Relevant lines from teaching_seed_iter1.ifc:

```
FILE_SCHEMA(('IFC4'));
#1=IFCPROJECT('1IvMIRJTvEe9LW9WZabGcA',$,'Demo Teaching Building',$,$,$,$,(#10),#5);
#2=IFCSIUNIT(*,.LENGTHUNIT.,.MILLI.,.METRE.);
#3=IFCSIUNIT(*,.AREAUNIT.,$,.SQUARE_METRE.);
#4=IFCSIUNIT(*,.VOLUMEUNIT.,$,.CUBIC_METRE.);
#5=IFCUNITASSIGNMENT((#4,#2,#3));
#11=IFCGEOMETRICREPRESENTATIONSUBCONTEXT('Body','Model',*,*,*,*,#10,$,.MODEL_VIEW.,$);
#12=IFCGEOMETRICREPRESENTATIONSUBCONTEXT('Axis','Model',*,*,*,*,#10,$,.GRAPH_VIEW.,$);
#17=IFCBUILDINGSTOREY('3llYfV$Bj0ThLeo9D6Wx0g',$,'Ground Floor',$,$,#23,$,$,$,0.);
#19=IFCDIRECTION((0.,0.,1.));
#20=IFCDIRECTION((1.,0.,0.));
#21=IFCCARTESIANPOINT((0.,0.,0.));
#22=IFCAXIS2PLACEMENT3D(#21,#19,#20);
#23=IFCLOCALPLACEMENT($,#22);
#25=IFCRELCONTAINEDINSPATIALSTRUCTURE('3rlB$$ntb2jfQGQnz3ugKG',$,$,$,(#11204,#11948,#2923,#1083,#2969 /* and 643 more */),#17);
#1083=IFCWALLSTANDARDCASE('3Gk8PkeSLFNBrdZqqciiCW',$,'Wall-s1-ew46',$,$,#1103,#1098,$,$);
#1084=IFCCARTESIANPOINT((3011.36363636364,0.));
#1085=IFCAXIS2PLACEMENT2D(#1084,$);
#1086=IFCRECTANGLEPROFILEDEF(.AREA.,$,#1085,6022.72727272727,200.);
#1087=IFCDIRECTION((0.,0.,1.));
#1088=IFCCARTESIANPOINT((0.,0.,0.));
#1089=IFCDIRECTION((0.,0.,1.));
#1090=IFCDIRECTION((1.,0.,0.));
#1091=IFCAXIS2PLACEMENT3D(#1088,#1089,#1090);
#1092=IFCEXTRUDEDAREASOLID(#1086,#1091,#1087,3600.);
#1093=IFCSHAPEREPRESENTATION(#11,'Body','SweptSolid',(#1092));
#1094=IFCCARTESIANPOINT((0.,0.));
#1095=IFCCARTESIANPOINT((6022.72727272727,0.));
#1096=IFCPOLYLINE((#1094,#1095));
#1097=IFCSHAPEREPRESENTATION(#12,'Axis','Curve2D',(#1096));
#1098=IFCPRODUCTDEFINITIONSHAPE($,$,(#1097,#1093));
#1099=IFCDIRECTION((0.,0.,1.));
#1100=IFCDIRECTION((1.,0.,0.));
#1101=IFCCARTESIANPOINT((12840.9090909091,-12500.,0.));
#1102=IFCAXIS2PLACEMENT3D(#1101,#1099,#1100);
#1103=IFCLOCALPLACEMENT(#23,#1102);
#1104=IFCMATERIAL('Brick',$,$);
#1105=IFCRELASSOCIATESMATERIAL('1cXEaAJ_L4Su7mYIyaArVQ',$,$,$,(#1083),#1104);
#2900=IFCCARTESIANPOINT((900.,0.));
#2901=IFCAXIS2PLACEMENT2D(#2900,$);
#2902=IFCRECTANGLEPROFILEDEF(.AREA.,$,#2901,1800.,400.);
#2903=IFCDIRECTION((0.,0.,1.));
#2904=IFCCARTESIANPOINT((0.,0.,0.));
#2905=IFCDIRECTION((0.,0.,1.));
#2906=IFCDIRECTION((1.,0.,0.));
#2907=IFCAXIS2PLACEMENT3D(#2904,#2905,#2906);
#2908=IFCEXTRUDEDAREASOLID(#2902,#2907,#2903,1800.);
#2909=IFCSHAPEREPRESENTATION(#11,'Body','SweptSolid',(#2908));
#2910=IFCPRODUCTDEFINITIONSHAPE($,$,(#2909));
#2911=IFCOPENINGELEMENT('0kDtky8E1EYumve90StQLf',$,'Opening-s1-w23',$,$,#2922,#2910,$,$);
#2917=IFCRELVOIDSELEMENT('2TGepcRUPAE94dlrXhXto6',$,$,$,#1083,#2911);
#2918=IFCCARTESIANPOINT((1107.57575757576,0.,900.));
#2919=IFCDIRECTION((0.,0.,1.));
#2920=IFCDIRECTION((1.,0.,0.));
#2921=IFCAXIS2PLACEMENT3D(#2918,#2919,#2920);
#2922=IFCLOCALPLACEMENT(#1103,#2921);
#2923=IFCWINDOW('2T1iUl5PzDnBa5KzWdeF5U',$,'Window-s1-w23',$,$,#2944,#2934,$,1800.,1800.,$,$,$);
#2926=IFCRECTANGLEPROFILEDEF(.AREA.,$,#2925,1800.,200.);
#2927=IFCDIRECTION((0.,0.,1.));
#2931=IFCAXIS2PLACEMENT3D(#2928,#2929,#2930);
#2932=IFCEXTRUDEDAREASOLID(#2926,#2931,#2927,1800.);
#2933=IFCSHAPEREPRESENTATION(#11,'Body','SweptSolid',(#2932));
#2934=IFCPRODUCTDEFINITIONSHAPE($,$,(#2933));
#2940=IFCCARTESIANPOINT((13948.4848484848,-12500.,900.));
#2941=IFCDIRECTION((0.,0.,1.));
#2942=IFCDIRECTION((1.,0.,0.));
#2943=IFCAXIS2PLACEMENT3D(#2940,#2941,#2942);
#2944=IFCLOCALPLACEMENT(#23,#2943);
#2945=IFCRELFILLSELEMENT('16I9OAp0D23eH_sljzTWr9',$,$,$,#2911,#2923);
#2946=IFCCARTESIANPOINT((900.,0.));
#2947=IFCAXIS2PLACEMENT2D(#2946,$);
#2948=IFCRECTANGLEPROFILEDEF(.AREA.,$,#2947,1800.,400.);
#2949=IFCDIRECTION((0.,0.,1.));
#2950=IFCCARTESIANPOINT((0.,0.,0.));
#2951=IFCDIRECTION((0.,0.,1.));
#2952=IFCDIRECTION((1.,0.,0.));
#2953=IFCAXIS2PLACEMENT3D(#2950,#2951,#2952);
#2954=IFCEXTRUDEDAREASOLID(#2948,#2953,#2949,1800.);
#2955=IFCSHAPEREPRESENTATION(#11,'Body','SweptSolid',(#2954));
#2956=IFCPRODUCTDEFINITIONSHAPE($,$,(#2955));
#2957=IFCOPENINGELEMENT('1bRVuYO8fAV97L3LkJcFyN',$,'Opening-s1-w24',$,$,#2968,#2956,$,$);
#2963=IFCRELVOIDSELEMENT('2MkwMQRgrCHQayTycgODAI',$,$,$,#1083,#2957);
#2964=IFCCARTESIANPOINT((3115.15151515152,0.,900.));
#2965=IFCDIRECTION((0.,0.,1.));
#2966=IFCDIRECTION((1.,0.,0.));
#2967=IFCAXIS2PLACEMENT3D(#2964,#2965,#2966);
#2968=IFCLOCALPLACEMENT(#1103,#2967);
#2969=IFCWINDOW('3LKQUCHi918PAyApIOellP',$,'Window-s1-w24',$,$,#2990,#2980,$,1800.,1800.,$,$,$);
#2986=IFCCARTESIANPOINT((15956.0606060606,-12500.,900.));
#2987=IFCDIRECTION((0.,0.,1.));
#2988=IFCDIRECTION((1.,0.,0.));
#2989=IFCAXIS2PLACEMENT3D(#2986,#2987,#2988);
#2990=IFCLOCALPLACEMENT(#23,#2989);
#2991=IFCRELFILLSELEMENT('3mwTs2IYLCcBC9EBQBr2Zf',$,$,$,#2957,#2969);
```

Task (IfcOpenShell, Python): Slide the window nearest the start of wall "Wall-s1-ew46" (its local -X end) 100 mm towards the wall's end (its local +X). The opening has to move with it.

```python
import ifcopenshell
import ifcopenshell.api.geometry
import ifcopenshell.util.placement
import ifcopenshell.util.unit

model = ifcopenshell.open("teaching_seed_iter1.ifc")
unit_scale = ifcopenshell.util.unit.calculate_unit_scale(model)

window = model.by_guid("2T1iUl5PzDnBa5KzWdeF5U")
opening = window.FillsVoids[0].RelatingOpeningElement
wall = opening.VoidsElements[0].RelatingBuildingElement

wall_matrix = ifcopenshell.util.placement.get_local_placement(wall.ObjectPlacement)
shift = wall_matrix[:3, 0] * 0.1 / unit_scale
before = ifcopenshell.util.placement.get_local_placement(window.ObjectPlacement)[:3, 3].copy()

# The window is not placed relative to its opening, so move both.
for product in (opening, window):
    matrix = ifcopenshell.util.placement.get_local_placement(product.ObjectPlacement)
    matrix[:3, 3] += shift
    ifcopenshell.api.geometry.edit_object_placement(model, product=product, matrix=matrix, is_si=False)

after = ifcopenshell.util.placement.get_local_placement(window.ObjectPlacement)[:3, 3]
print("window moved by", (after - before).round(3) + 0.0)

model.write("teaching_seed_iter1-out.ifc")
```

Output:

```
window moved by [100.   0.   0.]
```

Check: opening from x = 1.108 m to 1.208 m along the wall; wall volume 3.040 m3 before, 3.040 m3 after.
